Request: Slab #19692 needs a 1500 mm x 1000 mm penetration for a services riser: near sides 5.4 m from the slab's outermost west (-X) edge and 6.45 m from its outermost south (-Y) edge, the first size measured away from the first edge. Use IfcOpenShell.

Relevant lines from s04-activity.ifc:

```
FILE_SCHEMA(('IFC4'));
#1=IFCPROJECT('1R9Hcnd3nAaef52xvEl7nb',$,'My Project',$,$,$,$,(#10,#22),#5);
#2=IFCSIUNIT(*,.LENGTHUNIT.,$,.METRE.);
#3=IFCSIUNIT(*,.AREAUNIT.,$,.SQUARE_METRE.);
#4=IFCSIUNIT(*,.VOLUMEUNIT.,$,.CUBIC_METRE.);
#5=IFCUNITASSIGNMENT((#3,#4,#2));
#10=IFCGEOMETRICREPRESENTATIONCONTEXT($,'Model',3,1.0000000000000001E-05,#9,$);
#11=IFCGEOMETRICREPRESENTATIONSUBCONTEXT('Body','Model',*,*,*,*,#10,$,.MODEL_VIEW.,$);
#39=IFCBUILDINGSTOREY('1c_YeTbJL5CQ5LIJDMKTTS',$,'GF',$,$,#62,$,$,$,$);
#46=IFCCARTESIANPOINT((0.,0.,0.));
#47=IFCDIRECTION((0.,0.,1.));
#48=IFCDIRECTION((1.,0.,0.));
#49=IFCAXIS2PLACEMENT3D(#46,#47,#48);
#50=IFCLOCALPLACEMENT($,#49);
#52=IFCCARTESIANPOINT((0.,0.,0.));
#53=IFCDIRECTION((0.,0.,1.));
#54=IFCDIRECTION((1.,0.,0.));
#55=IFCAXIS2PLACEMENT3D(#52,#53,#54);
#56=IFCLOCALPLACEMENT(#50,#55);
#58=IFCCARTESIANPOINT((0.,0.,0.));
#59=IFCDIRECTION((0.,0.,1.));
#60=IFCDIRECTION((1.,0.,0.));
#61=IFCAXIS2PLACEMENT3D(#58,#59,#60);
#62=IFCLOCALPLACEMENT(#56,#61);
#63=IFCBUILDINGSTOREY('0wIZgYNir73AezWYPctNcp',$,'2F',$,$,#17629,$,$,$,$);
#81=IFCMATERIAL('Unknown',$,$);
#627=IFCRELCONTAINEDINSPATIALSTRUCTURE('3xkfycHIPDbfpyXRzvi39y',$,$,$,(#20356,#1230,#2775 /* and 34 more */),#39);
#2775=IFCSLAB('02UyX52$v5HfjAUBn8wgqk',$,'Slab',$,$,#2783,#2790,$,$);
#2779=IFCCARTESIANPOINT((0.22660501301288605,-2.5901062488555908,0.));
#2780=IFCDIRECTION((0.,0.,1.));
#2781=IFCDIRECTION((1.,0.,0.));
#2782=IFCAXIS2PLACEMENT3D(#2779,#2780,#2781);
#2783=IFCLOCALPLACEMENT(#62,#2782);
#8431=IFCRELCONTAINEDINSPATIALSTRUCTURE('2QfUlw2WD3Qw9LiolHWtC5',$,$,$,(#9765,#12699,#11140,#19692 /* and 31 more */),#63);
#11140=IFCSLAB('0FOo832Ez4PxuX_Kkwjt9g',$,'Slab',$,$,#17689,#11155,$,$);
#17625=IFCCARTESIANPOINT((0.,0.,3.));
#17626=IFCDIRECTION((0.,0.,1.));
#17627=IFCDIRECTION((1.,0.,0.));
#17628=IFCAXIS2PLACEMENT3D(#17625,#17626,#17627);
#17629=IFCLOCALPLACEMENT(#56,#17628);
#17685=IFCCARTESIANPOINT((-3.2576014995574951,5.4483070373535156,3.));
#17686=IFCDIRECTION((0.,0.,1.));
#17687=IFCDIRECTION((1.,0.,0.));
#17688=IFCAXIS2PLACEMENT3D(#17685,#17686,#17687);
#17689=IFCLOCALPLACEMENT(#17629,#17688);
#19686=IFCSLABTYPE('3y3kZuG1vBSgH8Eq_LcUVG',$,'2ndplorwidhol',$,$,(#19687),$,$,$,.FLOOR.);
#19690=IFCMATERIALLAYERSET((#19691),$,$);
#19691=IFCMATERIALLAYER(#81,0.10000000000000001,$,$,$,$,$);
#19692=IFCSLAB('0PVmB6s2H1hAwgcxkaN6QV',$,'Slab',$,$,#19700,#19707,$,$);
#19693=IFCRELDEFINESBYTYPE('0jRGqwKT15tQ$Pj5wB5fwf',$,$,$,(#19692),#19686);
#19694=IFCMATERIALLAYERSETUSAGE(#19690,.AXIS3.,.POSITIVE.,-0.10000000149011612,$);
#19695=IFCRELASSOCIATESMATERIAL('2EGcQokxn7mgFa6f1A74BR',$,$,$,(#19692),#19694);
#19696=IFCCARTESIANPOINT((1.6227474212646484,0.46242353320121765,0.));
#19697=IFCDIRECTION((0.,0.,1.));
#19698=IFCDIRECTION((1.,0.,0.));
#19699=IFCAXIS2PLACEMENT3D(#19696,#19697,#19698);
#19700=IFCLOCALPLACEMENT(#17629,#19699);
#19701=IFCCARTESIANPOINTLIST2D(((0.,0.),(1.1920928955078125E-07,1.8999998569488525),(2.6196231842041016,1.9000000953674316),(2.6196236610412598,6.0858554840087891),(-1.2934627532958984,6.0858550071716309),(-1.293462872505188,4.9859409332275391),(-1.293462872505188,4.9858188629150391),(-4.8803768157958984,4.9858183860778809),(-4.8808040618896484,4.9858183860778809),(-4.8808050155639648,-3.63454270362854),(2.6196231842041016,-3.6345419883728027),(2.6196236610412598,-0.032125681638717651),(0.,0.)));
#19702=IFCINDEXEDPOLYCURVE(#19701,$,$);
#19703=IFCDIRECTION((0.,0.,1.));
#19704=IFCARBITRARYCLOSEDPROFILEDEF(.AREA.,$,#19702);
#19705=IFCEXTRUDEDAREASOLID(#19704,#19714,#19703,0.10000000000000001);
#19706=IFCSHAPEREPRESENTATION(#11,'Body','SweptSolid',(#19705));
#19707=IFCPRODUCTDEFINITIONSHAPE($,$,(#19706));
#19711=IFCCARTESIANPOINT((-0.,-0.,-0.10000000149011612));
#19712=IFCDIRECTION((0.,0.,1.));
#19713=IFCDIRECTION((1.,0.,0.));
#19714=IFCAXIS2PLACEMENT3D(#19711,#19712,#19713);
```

```python
import numpy as np
import ifcopenshell
import ifcopenshell.api.feature
import ifcopenshell.api.geometry
import ifcopenshell.api.root
import ifcopenshell.geom
import ifcopenshell.util.placement
import ifcopenshell.util.representation
import ifcopenshell.util.shape
import ifcopenshell.util.unit

model = ifcopenshell.open("s04-activity.ifc")
unit_scale = ifcopenshell.util.unit.calculate_unit_scale(model)
settings = ifcopenshell.geom.settings()


def volume(element):
    """Net volume in cubic metres, openings subtracted."""
    shape = ifcopenshell.geom.create_shape(settings, element)
    return ifcopenshell.util.shape.get_volume(shape.geometry)


slab = model.by_guid("0PVmB6s2H1hAwgcxkaN6QV")
before = volume(slab)

# Extent in the slab's own axes, in metres. The edges named are its -X and -Y sides.
slab_shape = ifcopenshell.geom.create_shape(settings, slab)
vertices = ifcopenshell.util.shape.get_vertices(slab_shape.geometry)
x_min, y_min, bottom = vertices.min(axis=0)
top = vertices[:, 2].max()

opening = ifcopenshell.api.root.create_entity(model, ifc_class="IfcOpeningElement", name="Services riser opening", predefined_type="OPENING")
context = ifcopenshell.util.representation.get_context(model, "Model", "Body", "MODEL_VIEW")
width, depth = 1.5, 1
outline = [(0.0, 0.0), (width, 0.0), (width, depth), (0.0, depth), (0.0, 0.0)]
# Overshoot both faces by 50 mm so the cut is clean.
shape = ifcopenshell.api.geometry.add_slab_representation(
    model, context=context, depth=top - bottom + 0.1, polyline=outline
)
ifcopenshell.api.geometry.assign_representation(model, product=opening, representation=shape)

matrix = ifcopenshell.util.placement.get_local_placement(slab.ObjectPlacement)
matrix[:, 3] = matrix @ np.append(np.array([x_min + 5.4, y_min + 6.45, bottom - 0.05]) / unit_scale, 1.0)
ifcopenshell.api.geometry.edit_object_placement(model, product=opening, matrix=matrix, is_si=False)
ifcopenshell.api.feature.add_feature(model, feature=opening, element=slab)

after = volume(slab)

print(f"slab volume {before:.3f} -> {after:.3f} m3")

model.write("s04-activity-out.ifc")
```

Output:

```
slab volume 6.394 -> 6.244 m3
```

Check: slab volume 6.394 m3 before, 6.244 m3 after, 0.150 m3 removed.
